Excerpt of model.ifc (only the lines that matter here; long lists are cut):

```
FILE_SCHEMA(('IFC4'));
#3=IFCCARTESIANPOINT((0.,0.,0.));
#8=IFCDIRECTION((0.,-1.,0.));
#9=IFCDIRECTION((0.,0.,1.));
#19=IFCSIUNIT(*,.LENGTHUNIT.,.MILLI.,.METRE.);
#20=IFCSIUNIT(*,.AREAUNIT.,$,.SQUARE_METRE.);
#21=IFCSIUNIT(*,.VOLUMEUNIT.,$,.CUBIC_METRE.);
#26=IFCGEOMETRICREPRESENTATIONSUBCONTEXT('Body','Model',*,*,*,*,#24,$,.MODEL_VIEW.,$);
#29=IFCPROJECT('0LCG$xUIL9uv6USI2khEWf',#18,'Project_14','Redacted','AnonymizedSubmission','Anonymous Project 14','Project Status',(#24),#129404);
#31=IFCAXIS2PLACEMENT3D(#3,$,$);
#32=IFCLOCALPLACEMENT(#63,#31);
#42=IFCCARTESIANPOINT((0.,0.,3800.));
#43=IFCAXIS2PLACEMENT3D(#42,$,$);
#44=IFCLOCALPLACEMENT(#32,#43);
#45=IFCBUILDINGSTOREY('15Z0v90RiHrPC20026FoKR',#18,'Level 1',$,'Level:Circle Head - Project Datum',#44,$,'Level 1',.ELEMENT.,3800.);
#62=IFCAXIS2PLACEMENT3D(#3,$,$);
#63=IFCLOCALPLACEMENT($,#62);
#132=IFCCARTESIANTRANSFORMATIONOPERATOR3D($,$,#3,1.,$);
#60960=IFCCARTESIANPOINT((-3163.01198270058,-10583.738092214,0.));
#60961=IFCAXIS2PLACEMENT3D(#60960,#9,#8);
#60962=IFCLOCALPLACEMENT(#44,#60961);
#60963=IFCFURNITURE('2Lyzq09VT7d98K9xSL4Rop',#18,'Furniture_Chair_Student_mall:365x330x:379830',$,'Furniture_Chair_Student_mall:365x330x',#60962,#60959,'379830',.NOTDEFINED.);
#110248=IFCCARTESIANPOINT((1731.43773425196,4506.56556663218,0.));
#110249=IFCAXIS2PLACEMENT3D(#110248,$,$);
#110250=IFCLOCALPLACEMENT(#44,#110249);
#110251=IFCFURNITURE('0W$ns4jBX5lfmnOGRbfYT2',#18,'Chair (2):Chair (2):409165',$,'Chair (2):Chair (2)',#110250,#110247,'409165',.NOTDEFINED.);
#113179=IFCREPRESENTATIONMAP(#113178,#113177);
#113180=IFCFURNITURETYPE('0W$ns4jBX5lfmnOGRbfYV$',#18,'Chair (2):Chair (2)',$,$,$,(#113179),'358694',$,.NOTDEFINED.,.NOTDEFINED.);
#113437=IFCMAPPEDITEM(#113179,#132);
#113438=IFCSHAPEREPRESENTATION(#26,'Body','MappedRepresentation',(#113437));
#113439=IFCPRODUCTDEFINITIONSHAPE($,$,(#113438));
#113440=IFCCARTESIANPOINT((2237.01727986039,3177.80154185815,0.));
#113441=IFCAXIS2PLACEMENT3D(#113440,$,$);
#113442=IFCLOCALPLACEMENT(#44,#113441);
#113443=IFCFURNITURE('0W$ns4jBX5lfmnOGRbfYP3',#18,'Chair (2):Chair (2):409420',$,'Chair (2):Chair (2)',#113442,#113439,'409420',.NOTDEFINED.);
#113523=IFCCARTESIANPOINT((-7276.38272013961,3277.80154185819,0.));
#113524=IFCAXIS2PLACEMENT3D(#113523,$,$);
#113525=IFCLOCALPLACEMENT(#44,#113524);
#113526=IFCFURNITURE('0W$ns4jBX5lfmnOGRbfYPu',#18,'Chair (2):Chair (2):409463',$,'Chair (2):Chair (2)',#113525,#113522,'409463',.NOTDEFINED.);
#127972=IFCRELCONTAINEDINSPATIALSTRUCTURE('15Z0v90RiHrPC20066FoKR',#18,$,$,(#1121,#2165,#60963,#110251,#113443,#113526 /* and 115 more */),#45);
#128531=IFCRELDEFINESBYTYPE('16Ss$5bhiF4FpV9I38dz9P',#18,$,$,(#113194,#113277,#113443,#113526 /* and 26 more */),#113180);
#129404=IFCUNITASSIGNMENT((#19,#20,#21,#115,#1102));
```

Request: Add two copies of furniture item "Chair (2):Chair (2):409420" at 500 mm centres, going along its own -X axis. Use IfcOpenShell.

```python
import ifcopenshell
import ifcopenshell.api.geometry
import ifcopenshell.api.root
import ifcopenshell.util.element
import ifcopenshell.util.placement

model = ifcopenshell.open("model.ifc")


def reuse_history(source, copy):
    """copy_class also copies each property set's owner history, people and application; keep the originals."""
    for rel in copy.IsDefinedBy:
        if rel.is_a("IfcRelDefinesByProperties") and (history := rel.RelatingPropertyDefinition.OwnerHistory):
            rel.RelatingPropertyDefinition.OwnerHistory = source.OwnerHistory
            ifcopenshell.util.element.remove_deep2(model, history)


source = model.by_guid("0W$ns4jBX5lfmnOGRbfYP3")
base = ifcopenshell.util.placement.get_local_placement(source.ObjectPlacement)
step = -base[:3, 0] * 500.0

for i in range(1, 3):
    copy = ifcopenshell.api.root.copy_class(model, product=source)
    copy.Representation = ifcopenshell.util.element.copy_deep(
        model, source.Representation, exclude=["IfcGeometricRepresentationContext", "IfcRepresentationMap"]
    )
    copy.Name = "Chair (2):Chair (2)"
    copy.Tag = None
    reuse_history(source, copy)
    matrix = base.copy()
    matrix[:3, 3] += i * step
    print("added at", matrix[:3, 3].round(3) + 0.0)
    ifcopenshell.api.geometry.edit_object_placement(model, product=copy, matrix=matrix, is_si=False)

model.write("model_updated.ifc")
```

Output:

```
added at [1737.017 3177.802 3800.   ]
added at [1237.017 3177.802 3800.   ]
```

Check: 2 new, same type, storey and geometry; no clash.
